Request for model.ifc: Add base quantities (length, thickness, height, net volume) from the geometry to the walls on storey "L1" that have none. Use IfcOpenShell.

First a look at what the model holds.

```python
import ifcopenshell
import ifcopenshell.util.element
import ifcopenshell.util.unit

model = ifcopenshell.open("model.ifc")
print(model.schema)
for unit_type in ("LENGTHUNIT", "AREAUNIT", "VOLUMEUNIT"):
    print(unit_type, ifcopenshell.util.unit.calculate_unit_scale(model, unit_type))
storey = next(s for s in model.by_type("IfcBuildingStorey") if s.Name == "L1")
walls = [e for e in ifcopenshell.util.element.get_decomposition(storey) if e.is_a("IfcWall")]
for e in sorted(walls, key=lambda e: e.id()):
    print(e.id(), e.is_a(), e.Name, list(ifcopenshell.util.element.get_psets(e, qtos_only=True)), sep=" | ")
```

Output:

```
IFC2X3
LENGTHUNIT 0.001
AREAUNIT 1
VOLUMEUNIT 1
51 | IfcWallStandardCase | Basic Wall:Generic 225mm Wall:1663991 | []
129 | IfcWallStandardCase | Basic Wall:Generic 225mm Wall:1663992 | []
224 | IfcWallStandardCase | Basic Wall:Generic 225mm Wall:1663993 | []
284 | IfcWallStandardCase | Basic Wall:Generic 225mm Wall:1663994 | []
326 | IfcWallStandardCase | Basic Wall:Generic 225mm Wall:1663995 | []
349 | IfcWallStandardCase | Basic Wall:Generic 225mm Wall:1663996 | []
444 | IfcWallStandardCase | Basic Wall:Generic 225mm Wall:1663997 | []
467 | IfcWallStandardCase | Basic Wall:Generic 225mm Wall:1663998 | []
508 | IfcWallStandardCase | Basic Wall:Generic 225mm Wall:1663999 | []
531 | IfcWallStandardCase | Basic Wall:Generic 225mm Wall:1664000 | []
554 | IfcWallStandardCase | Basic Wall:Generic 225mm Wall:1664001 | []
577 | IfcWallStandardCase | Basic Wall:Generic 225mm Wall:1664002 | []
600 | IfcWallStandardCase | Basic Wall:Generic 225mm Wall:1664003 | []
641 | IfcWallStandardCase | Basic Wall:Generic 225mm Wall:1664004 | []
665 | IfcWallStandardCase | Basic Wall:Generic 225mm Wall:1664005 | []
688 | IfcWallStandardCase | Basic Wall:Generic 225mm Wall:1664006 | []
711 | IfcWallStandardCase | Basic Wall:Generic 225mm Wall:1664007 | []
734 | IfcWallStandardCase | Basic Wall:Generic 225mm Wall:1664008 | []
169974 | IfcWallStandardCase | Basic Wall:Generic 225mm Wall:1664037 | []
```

```python
import ifcopenshell
import ifcopenshell.api.pset
import ifcopenshell.geom
import ifcopenshell.util.element
import ifcopenshell.util.shape
import ifcopenshell.util.unit

model = ifcopenshell.open("model.ifc")
unit_scale = ifcopenshell.util.unit.calculate_unit_scale(model)
volume_scale = ifcopenshell.util.unit.calculate_unit_scale(model, "VOLUMEUNIT")
settings = ifcopenshell.geom.settings()

storey = next(s for s in model.by_type("IfcBuildingStorey") if s.Name == "L1")
walls = [e for e in ifcopenshell.util.element.get_decomposition(storey) if e.is_a("IfcWall")]

for e in sorted(walls, key=lambda e: e.id()):
    if ifcopenshell.util.element.get_psets(e, qtos_only=True, should_inherit=False):
        continue
    # Geometry comes back in metres, in the element's own axes.
    shape = ifcopenshell.geom.create_shape(settings, e)
    values = {
        "Length": ifcopenshell.util.shape.get_x(shape.geometry) / unit_scale,
        "Width": ifcopenshell.util.shape.get_y(shape.geometry) / unit_scale,
        "Height": ifcopenshell.util.shape.get_z(shape.geometry) / unit_scale,
        "NetVolume": ifcopenshell.util.shape.get_volume(shape.geometry) / volume_scale,
    }
    qto = ifcopenshell.api.pset.add_qto(model, product=e, name="BaseQuantities")
    ifcopenshell.api.pset.edit_qto(model, qto=qto, properties=values)
    print(e.id(), {k: round(v, 3) for k, v in values.items()})

model.write("model_rev.ifc")
```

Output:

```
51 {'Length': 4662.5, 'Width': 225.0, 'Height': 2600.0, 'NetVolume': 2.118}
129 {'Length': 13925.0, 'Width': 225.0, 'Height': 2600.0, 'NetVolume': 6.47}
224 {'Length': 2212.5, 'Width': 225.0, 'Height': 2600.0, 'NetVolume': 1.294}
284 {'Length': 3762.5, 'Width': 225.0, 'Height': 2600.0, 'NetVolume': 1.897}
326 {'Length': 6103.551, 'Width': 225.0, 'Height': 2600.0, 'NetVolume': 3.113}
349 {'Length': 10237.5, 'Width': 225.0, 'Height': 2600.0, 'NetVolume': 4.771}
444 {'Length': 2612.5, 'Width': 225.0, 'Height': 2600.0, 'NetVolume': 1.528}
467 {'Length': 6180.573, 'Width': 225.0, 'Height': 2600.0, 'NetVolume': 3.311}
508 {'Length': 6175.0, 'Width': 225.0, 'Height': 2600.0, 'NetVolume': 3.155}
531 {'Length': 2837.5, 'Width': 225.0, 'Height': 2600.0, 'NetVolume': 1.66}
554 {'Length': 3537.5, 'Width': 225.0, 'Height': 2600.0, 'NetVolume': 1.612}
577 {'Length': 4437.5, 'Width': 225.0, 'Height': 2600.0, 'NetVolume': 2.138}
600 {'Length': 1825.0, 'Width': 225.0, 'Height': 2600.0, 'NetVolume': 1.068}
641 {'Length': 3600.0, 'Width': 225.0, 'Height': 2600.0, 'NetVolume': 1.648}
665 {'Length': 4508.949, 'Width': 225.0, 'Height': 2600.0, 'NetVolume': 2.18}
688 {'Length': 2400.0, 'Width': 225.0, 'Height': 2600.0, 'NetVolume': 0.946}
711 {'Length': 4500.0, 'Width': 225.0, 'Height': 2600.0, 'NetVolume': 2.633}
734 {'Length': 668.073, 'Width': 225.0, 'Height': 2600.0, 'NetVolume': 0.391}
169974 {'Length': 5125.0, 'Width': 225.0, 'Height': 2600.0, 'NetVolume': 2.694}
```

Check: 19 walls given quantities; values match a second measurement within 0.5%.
